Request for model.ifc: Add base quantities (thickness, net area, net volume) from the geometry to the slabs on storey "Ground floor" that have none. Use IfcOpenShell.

First a look at what the model holds.

```python
import ifcopenshell
import ifcopenshell.util.element
import ifcopenshell.util.unit

model = ifcopenshell.open("model.ifc")
print(model.schema)
for unit_type in ("LENGTHUNIT", "AREAUNIT", "VOLUMEUNIT"):
    print(unit_type, ifcopenshell.util.unit.calculate_unit_scale(model, unit_type))
storey = next(s for s in model.by_type("IfcBuildingStorey") if s.Name == "Ground floor")
slabs = [e for e in ifcopenshell.util.element.get_decomposition(storey) if e.is_a("IfcSlab")]
for e in sorted(slabs, key=lambda e: e.id()):
    print(e.id(), e.is_a(), e.Name, list(ifcopenshell.util.element.get_psets(e, qtos_only=True)), sep=" | ")
```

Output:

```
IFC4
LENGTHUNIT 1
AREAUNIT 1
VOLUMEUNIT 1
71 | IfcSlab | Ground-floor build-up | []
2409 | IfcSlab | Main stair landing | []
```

```python
import ifcopenshell
import ifcopenshell.api.pset
import ifcopenshell.geom
import ifcopenshell.util.element
import ifcopenshell.util.shape
import ifcopenshell.util.unit

model = ifcopenshell.open("model.ifc")
unit_scale = ifcopenshell.util.unit.calculate_unit_scale(model)
area_scale = ifcopenshell.util.unit.calculate_unit_scale(model, "AREAUNIT")
volume_scale = ifcopenshell.util.unit.calculate_unit_scale(model, "VOLUMEUNIT")
settings = ifcopenshell.geom.settings()

storey = next(s for s in model.by_type("IfcBuildingStorey") if s.Name == "Ground floor")
slabs = [e for e in ifcopenshell.util.element.get_decomposition(storey) if e.is_a("IfcSlab")]

for e in sorted(slabs, key=lambda e: e.id()):
    if ifcopenshell.util.element.get_psets(e, qtos_only=True, should_inherit=False):
        continue
    # Geometry comes back in metres, in the element's own axes.
    shape = ifcopenshell.geom.create_shape(settings, e)
    values = {
        "Width": ifcopenshell.util.shape.get_z(shape.geometry) / unit_scale,
        "NetArea": ifcopenshell.util.shape.get_footprint_area(shape.geometry) / area_scale,
        "NetVolume": ifcopenshell.util.shape.get_volume(shape.geometry) / volume_scale,
    }
    qto = ifcopenshell.api.pset.add_qto(model, product=e, name="Qto_SlabBaseQuantities")
    ifcopenshell.api.pset.edit_qto(model, qto=qto, properties=values)
    print(e.id(), {k: round(v, 3) for k, v in values.items()})

model.write("model-out.ifc")
```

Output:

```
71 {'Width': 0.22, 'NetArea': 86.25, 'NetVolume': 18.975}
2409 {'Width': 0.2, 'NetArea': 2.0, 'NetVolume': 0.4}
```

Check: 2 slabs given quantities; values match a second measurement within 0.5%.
